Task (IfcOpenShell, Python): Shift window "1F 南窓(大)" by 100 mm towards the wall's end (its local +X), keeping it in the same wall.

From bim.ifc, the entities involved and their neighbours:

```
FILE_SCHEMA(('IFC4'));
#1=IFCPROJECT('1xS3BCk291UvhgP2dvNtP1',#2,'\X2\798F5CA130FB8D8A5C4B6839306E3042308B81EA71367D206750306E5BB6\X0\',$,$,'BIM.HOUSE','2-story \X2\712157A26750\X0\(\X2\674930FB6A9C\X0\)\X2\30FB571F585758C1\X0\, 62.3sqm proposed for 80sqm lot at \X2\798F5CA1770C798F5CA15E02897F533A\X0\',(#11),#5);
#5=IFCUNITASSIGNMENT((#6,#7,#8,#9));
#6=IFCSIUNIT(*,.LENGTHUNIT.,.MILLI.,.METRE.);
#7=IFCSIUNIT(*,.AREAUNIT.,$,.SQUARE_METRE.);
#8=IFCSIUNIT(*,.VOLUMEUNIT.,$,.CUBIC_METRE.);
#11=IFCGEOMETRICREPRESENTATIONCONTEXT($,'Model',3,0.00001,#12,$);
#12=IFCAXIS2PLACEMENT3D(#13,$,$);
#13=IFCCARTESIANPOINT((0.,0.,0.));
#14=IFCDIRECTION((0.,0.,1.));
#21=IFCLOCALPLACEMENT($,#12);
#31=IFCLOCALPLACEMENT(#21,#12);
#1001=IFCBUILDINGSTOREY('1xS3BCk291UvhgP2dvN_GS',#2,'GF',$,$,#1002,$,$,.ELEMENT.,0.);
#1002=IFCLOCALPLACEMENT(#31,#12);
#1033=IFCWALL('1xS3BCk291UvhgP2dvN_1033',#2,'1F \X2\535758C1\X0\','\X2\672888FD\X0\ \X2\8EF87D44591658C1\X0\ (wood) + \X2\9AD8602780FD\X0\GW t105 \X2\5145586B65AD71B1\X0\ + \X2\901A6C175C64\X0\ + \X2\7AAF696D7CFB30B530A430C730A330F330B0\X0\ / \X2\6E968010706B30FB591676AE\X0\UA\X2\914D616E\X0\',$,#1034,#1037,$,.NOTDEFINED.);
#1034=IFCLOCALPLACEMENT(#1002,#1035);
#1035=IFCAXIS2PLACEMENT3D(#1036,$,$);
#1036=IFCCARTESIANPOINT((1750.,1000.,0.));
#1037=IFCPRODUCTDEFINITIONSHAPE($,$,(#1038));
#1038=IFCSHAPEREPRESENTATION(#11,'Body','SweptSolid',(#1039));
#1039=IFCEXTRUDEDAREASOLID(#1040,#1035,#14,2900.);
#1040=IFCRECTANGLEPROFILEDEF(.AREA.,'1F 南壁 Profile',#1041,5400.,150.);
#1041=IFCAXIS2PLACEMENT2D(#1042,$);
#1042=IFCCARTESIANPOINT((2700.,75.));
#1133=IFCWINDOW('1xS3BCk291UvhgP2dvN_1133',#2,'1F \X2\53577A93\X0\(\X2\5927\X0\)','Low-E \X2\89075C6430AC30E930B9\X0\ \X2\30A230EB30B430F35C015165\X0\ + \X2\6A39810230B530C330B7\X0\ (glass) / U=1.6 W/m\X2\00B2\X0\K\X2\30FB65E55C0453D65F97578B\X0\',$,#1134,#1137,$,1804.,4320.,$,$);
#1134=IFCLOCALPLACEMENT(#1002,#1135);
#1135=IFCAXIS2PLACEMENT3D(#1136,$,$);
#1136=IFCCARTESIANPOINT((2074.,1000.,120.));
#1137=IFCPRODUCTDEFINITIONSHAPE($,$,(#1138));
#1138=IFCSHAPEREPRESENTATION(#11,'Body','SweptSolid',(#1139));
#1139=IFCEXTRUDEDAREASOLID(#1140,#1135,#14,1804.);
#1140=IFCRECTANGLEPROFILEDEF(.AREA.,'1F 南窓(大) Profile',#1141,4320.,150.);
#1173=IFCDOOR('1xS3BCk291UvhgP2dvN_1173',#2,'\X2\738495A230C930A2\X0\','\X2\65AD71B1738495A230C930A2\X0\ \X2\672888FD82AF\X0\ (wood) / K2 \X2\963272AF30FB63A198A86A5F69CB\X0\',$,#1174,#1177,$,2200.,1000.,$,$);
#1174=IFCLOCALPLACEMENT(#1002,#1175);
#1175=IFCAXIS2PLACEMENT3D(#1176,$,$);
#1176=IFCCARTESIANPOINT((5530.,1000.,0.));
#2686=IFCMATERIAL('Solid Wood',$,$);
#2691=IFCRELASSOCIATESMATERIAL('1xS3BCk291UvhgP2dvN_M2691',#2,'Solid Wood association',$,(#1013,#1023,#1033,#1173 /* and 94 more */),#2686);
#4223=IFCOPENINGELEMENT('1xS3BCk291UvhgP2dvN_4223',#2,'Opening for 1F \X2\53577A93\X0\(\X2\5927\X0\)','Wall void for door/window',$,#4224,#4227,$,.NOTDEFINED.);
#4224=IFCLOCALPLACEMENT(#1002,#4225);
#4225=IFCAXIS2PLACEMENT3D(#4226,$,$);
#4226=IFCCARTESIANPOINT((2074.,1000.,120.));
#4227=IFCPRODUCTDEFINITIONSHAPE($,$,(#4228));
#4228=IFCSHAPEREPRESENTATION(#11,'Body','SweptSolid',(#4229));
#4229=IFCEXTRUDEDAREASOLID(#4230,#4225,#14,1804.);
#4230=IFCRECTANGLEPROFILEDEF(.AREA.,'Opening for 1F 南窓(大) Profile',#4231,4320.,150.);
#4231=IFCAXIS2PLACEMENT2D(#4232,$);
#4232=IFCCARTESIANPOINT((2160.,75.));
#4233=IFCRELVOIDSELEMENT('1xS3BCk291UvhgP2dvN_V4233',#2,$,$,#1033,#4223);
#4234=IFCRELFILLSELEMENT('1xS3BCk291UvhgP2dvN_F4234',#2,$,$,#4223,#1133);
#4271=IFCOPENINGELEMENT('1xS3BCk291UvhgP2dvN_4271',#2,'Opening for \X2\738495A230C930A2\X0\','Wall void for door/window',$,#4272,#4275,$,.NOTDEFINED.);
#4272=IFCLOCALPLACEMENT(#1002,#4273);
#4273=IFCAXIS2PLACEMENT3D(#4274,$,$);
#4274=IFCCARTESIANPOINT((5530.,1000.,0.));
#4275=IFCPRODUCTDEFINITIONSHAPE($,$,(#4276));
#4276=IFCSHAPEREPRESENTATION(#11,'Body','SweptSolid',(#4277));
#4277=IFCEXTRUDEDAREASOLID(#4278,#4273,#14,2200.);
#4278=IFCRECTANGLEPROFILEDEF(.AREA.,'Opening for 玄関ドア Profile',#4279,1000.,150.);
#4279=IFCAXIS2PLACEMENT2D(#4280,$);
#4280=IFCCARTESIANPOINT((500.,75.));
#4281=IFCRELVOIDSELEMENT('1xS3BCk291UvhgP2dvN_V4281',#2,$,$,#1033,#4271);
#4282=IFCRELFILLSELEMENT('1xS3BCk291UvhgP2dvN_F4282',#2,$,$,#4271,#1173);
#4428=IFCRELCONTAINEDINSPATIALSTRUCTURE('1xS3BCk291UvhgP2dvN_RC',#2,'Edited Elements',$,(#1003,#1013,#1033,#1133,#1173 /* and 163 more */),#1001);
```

```python
import ifcopenshell
import ifcopenshell.api.geometry
import ifcopenshell.util.placement
import ifcopenshell.util.unit

model = ifcopenshell.open("bim.ifc")
unit_scale = ifcopenshell.util.unit.calculate_unit_scale(model)

window = model.by_guid("1xS3BCk291UvhgP2dvN_1133")
opening = window.FillsVoids[0].RelatingOpeningElement
wall = opening.VoidsElements[0].RelatingBuildingElement

wall_matrix = ifcopenshell.util.placement.get_local_placement(wall.ObjectPlacement)
shift = wall_matrix[:3, 0] * 0.1 / unit_scale
before = ifcopenshell.util.placement.get_local_placement(window.ObjectPlacement)[:3, 3].copy()

# The window is not placed relative to its opening, so move both.
for product in (opening, window):
    matrix = ifcopenshell.util.placement.get_local_placement(product.ObjectPlacement)
    matrix[:3, 3] += shift
    ifcopenshell.api.geometry.edit_object_placement(model, product=product, matrix=matrix, is_si=False)

after = ifcopenshell.util.placement.get_local_placement(window.ObjectPlacement)[:3, 3]
print("window moved by", (after - before).round(3) + 0.0)

model.write("bim_v2.ifc")
```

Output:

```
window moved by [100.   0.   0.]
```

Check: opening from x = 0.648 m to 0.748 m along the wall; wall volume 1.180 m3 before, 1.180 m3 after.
